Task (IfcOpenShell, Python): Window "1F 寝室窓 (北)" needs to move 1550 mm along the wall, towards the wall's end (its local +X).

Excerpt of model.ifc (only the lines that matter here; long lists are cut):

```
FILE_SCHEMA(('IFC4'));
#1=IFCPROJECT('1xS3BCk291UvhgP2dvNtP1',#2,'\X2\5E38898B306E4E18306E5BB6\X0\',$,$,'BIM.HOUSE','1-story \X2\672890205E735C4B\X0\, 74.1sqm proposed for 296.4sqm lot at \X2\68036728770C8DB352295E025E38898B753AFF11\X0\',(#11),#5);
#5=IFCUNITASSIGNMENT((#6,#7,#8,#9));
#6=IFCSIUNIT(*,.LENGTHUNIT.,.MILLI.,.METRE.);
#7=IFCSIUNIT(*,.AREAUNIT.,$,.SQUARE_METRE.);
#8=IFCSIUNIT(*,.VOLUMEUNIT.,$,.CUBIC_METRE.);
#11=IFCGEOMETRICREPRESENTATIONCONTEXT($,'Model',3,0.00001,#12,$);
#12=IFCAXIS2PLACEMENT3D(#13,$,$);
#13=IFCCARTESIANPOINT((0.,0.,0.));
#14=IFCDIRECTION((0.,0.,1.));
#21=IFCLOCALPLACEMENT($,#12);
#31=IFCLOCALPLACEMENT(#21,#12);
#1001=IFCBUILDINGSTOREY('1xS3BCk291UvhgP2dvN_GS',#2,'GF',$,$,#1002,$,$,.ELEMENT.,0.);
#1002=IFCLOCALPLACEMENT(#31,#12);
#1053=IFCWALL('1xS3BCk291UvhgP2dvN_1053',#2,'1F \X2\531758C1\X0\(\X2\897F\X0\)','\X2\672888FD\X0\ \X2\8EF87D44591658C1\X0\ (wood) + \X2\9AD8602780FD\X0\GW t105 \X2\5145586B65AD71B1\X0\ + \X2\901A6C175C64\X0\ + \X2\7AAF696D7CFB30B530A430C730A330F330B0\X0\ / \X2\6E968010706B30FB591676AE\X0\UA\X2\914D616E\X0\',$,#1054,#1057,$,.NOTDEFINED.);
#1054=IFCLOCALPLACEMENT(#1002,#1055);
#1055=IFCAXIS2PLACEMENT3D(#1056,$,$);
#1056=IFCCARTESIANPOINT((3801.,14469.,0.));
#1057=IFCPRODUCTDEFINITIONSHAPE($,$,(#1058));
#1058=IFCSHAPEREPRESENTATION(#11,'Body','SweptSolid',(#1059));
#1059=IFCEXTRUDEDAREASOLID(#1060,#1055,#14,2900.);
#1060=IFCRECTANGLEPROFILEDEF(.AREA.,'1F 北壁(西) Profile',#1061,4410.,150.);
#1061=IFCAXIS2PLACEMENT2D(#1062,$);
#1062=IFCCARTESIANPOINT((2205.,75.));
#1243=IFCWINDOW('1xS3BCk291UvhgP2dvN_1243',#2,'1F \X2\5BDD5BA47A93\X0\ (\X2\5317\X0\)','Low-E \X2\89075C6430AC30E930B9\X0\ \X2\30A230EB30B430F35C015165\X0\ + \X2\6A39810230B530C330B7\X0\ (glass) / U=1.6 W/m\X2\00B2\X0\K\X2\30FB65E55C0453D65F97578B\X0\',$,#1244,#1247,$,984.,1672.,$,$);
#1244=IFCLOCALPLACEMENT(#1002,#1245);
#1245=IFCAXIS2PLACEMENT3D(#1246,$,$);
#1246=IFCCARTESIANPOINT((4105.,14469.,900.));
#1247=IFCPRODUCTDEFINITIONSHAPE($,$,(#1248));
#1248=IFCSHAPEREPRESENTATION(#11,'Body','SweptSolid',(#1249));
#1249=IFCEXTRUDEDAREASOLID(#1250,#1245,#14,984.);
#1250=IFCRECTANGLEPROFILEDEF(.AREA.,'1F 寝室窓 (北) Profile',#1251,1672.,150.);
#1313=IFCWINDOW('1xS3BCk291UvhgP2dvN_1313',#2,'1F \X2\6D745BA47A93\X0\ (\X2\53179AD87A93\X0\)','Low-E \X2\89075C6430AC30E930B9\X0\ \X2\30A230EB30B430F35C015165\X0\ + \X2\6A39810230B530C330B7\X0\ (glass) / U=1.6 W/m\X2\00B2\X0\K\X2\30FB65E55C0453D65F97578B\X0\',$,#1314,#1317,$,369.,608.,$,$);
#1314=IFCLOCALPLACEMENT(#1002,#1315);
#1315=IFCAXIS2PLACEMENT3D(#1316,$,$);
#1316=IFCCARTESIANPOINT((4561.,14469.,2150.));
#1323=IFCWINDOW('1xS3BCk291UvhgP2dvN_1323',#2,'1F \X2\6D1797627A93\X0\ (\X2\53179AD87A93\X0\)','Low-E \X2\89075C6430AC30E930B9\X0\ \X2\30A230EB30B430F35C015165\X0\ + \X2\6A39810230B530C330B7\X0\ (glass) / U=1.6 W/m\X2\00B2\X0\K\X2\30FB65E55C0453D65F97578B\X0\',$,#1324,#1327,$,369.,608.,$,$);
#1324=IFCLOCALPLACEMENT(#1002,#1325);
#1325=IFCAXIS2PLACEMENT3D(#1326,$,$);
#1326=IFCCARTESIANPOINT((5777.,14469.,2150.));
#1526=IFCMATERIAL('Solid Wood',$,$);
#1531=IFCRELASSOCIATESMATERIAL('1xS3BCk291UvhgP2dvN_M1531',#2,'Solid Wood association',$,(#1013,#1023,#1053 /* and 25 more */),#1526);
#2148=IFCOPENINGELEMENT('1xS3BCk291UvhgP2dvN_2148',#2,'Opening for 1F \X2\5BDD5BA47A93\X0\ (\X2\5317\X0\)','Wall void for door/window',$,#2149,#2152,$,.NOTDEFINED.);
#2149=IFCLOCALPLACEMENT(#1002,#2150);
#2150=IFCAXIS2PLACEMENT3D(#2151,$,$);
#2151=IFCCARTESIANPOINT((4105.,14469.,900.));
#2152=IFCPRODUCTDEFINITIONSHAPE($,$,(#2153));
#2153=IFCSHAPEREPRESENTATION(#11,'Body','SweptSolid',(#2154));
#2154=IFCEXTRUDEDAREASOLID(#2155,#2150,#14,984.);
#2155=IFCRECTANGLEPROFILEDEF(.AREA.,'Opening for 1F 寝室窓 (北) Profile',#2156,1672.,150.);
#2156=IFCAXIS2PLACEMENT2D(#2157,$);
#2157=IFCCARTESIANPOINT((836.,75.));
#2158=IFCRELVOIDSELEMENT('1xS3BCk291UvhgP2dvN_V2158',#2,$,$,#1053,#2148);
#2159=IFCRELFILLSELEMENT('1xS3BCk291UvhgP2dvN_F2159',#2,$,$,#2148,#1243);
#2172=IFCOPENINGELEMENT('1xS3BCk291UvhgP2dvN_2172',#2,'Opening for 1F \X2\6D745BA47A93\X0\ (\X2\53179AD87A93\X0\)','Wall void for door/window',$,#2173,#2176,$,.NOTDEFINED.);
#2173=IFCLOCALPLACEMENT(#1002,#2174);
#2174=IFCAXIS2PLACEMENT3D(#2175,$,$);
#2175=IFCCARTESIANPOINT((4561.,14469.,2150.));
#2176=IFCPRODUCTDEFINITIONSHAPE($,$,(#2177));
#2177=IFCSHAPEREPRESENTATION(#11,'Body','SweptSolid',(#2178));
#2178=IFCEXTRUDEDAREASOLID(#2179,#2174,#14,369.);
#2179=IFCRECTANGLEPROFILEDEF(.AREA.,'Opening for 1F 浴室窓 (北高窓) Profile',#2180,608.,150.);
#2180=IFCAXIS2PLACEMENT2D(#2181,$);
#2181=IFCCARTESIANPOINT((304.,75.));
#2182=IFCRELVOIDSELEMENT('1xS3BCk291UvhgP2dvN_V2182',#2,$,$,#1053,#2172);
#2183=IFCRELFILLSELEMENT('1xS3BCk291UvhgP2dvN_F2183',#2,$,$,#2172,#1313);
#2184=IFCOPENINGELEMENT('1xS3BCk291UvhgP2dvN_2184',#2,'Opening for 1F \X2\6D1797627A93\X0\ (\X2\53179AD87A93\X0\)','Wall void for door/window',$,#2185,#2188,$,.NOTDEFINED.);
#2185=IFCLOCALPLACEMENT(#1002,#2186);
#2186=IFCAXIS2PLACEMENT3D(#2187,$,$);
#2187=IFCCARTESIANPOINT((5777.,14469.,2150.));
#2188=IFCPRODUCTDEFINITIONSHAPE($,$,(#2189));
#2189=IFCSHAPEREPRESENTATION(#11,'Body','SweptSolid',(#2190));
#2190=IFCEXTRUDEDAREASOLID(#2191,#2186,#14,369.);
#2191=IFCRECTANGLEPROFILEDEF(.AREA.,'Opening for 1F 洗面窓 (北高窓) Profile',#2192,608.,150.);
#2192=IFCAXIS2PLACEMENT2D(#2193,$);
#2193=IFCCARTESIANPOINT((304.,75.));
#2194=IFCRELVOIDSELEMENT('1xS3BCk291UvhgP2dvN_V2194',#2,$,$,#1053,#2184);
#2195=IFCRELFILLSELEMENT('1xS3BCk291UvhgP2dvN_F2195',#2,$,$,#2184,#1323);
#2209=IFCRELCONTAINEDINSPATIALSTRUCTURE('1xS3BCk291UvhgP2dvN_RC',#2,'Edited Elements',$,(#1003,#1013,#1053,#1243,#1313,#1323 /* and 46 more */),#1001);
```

```python
import ifcopenshell
import ifcopenshell.api.geometry
import ifcopenshell.util.placement
import ifcopenshell.util.unit

model = ifcopenshell.open("model.ifc")
unit_scale = ifcopenshell.util.unit.calculate_unit_scale(model)

window = model.by_guid("1xS3BCk291UvhgP2dvN_1243")
opening = window.FillsVoids[0].RelatingOpeningElement
wall = opening.VoidsElements[0].RelatingBuildingElement

wall_matrix = ifcopenshell.util.placement.get_local_placement(wall.ObjectPlacement)
shift = wall_matrix[:3, 0] * 1.55 / unit_scale
before = ifcopenshell.util.placement.get_local_placement(window.ObjectPlacement)[:3, 3].copy()

# The window is not placed relative to its opening, so move both.
for product in (opening, window):
    matrix = ifcopenshell.util.placement.get_local_placement(product.ObjectPlacement)
    matrix[:3, 3] += shift
    ifcopenshell.api.geometry.edit_object_placement(model, product=product, matrix=matrix, is_si=False)

after = ifcopenshell.util.placement.get_local_placement(window.ObjectPlacement)[:3, 3]
print("window moved by", (after - before).round(3) + 0.0)

model.write("model_v2.ifc")
```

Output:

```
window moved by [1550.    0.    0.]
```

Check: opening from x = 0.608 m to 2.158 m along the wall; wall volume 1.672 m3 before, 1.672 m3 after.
